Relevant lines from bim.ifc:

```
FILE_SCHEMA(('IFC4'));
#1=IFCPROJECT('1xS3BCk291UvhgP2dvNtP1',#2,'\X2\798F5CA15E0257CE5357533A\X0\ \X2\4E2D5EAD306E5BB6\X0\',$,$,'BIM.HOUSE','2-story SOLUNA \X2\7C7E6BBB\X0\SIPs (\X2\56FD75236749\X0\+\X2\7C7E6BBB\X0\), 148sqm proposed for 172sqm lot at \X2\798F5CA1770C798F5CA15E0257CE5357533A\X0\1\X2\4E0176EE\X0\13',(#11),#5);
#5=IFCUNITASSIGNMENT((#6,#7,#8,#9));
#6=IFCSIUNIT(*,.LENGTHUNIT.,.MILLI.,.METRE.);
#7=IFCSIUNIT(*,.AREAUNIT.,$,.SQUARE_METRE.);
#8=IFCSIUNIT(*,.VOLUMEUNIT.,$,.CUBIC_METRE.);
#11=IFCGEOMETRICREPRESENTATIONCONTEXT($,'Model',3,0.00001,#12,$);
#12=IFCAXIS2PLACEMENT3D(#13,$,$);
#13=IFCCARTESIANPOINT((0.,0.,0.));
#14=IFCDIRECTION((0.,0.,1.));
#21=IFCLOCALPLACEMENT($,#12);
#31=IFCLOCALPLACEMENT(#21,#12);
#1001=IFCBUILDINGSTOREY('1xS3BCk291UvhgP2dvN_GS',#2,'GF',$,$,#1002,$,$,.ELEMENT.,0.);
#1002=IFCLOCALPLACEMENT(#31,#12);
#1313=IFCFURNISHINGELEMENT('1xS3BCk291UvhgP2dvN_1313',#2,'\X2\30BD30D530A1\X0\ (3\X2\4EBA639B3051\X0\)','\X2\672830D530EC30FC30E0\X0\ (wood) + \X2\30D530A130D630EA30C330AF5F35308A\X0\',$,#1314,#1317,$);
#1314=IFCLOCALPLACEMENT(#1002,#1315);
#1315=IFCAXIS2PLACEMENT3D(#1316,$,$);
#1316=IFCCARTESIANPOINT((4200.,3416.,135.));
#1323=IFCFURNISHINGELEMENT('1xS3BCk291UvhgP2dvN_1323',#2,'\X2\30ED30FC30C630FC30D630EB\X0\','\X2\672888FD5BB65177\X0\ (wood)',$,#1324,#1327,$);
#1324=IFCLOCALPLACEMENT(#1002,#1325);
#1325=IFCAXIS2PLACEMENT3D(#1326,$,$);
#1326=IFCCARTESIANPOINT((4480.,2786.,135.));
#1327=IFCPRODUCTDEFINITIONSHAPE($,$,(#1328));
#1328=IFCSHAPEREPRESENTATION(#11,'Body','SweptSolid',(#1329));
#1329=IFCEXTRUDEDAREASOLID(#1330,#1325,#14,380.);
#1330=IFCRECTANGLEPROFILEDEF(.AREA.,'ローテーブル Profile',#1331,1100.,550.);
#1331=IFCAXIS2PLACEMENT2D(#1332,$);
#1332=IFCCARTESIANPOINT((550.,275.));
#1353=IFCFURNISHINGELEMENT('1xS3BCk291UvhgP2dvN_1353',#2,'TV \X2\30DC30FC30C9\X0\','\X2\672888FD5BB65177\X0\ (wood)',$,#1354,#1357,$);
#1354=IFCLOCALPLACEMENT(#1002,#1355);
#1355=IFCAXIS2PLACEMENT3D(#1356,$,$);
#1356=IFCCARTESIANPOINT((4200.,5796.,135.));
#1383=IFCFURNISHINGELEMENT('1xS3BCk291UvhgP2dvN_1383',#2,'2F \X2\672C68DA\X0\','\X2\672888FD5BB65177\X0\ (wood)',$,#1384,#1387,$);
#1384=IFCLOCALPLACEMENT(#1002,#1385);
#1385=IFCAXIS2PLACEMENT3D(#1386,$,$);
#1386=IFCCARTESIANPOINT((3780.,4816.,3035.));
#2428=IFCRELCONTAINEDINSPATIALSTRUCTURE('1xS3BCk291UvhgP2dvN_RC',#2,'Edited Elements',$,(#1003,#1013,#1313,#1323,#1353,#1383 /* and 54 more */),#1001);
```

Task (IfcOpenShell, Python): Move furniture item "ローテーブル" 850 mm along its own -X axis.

```python
import ifcopenshell
import ifcopenshell.api.geometry
import ifcopenshell.util.placement
import ifcopenshell.util.unit

model = ifcopenshell.open("bim.ifc")
unit_scale = ifcopenshell.util.unit.calculate_unit_scale(model)

item = model.by_guid("1xS3BCk291UvhgP2dvN_1323")
matrix = ifcopenshell.util.placement.get_local_placement(item.ObjectPlacement)
matrix[:3, 3] -= matrix[:3, 0] * 0.85 / unit_scale
ifcopenshell.api.geometry.edit_object_placement(model, product=item, matrix=matrix, is_si=False)

print(ifcopenshell.util.placement.get_local_placement(item.ObjectPlacement).round(3) + 0.0)

model.write("bim_v2.ifc")
```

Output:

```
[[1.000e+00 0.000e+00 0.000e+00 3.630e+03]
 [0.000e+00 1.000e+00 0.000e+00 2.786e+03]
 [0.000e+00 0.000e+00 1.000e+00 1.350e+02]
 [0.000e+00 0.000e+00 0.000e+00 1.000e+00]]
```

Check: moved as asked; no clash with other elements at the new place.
